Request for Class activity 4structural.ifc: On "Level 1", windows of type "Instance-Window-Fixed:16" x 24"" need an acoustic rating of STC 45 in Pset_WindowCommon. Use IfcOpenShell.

First a look at what the model holds.

```python
import ifcopenshell
import ifcopenshell.util.element

model = ifcopenshell.open("Class activity 4structural.ifc")
print(model.schema)
storey = next(s for s in model.by_type("IfcBuildingStorey") if s.Name == "Level 1")
windows = [e for e in ifcopenshell.util.element.get_decomposition(storey) if e.is_a("IfcWindow")]
seen = {}
for e in windows:
    element_type = ifcopenshell.util.element.get_type(e)
    key = (element_type.Name if element_type != e and element_type else None, ifcopenshell.util.element.get_pset(e, "Pset_WindowCommon", "AcousticRating"))
    seen[key] = seen.get(key, 0) + 1
for (name, value), count in sorted(seen.items(), key=str):
    print(count, "x", name, "|", value)
```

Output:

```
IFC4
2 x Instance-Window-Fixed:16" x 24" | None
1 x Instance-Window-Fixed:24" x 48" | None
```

```python
import ifcopenshell
import ifcopenshell.api.pset
import ifcopenshell.util.element

model = ifcopenshell.open("Class activity 4structural.ifc")

storey = next(s for s in model.by_type("IfcBuildingStorey") if s.Name == "Level 1")
windows = [e for e in ifcopenshell.util.element.get_decomposition(storey) if e.is_a("IfcWindow")]

count = 0
for e in windows:
    element_type = ifcopenshell.util.element.get_type(e)
    if element_type in (None, e) or element_type.Name != 'Instance-Window-Fixed:16" x 24"':
        continue
    # add_pset returns the element's existing set when there is one.
    pset = ifcopenshell.api.pset.add_pset(model, product=e, name="Pset_WindowCommon")
    ifcopenshell.api.pset.edit_pset(model, pset=pset, properties={"AcousticRating": "STC 45"})
    count += 1

print(count, "windows updated")

model.write("Class activity 4structural_v2.ifc")
```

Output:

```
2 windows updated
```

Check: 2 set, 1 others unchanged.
